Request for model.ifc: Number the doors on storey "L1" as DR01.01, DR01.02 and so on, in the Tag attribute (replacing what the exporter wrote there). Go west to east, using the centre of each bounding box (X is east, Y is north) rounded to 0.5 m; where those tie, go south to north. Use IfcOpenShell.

First a look at what the model holds.

```python
import ifcopenshell
import ifcopenshell.util.element
import ifcopenshell.util.placement

model = ifcopenshell.open("model.ifc")
print(model.schema)
storey = next(s for s in model.by_type("IfcBuildingStorey") if s.Name == "L1")
doors = [e for e in ifcopenshell.util.element.get_decomposition(storey) if e.is_a("IfcDoor")]
for e in sorted(doors, key=lambda e: e.id()):
    origin = ifcopenshell.util.placement.get_local_placement(e.ObjectPlacement)[:3, 3]
    print(e.id(), e.Tag, e.Name, origin.round(2) + 0.0, sep=" | ")
```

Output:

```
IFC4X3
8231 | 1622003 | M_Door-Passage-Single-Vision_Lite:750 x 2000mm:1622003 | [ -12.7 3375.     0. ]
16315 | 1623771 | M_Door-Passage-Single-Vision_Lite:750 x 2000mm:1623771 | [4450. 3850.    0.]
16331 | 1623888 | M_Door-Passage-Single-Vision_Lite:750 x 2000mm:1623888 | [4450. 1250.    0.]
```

```python
import ifcopenshell
import ifcopenshell.geom
import ifcopenshell.util.element
import ifcopenshell.util.shape

model = ifcopenshell.open("model.ifc")
settings = ifcopenshell.geom.settings()
settings.set("use-world-coords", True)


def centre(element):
    shape = ifcopenshell.geom.create_shape(settings, element)
    return ifcopenshell.util.shape.get_bbox_centroid(shape.geometry)


storey = next(s for s in model.by_type("IfcBuildingStorey") if s.Name == "L1")
doors = [e for e in ifcopenshell.util.element.get_decomposition(storey) if e.is_a("IfcDoor")]

# Insertion points can sit at a corner or the storey origin, so sort by the geometry (in metres).
centres = {e: centre(e) for e in doors}
doors.sort(key=lambda e: (round(centres[e][0] / 0.5), centres[e][1]))

for i, e in enumerate(doors, start=1):
    number = f"DR01.{i:02d}"
    e.Tag = number
    print(e.id(), number)

model.write("model-out.ifc")
```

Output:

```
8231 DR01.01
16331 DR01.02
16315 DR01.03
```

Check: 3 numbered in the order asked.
